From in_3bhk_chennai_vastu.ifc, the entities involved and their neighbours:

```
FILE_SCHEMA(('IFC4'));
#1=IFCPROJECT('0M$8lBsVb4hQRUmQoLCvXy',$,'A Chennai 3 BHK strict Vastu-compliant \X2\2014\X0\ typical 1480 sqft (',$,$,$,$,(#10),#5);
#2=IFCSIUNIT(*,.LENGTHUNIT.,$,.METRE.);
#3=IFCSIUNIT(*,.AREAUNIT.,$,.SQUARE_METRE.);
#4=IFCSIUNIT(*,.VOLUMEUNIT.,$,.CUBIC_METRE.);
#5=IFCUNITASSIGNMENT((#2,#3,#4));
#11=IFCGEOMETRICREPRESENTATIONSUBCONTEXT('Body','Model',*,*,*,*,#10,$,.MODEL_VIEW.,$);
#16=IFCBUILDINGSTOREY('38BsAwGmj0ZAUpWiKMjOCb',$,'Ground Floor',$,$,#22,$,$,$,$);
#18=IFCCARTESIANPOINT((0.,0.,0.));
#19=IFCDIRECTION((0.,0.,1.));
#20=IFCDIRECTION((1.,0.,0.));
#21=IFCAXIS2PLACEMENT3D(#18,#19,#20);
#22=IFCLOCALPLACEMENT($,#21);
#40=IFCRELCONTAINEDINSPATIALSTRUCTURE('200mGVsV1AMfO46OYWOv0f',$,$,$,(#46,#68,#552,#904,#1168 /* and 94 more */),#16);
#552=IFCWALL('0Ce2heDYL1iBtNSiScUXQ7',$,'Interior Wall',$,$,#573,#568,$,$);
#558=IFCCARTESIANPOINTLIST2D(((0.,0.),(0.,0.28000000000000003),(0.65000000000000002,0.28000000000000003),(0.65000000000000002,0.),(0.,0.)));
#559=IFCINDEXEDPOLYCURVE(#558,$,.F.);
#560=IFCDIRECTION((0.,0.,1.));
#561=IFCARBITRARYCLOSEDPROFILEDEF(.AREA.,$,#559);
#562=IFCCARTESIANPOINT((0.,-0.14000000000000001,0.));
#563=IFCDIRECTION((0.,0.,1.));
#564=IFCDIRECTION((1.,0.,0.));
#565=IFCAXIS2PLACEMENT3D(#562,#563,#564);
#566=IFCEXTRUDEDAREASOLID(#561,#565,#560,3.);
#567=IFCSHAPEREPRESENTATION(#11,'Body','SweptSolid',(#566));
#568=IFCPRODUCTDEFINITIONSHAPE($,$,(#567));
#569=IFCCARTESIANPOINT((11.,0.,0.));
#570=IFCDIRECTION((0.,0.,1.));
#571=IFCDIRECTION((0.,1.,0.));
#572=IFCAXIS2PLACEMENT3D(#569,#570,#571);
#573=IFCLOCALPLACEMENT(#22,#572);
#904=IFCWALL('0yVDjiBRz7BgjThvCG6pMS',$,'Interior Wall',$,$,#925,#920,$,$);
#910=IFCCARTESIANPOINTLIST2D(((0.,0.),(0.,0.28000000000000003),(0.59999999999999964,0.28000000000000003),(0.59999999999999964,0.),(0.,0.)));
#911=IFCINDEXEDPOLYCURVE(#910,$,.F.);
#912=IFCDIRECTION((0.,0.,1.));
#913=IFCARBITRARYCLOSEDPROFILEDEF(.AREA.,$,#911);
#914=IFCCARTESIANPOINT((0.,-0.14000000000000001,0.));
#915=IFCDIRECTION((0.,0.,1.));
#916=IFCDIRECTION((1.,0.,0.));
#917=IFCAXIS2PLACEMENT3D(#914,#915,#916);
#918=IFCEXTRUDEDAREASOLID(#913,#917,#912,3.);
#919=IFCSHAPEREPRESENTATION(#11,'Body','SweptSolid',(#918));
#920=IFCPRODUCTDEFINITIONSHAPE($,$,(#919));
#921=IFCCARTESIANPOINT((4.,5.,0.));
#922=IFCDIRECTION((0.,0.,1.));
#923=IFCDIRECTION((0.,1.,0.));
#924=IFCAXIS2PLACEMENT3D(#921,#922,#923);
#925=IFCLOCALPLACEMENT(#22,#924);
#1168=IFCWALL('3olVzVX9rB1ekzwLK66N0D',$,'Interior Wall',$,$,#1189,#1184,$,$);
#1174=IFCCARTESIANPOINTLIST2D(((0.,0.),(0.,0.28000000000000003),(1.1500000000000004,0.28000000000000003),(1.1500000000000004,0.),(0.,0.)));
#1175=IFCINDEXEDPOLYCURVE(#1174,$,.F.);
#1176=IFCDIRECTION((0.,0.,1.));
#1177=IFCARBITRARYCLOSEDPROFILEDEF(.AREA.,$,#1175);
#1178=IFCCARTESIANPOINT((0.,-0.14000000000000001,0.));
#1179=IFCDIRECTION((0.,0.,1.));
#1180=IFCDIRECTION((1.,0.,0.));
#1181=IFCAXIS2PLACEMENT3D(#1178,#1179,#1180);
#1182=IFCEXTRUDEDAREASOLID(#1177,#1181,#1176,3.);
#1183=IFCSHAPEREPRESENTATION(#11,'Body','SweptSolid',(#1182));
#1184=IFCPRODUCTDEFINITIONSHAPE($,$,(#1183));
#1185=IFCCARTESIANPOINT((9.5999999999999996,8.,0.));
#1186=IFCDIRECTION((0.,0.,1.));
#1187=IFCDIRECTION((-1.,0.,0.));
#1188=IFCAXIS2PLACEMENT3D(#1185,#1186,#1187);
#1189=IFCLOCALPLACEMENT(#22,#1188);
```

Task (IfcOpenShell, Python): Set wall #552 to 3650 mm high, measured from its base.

```python
import ifcopenshell
import ifcopenshell.geom
import ifcopenshell.util.representation
import ifcopenshell.util.shape
import ifcopenshell.util.unit

model = ifcopenshell.open("in_3bhk_chennai_vastu.ifc")
unit_scale = ifcopenshell.util.unit.calculate_unit_scale(model)
settings = ifcopenshell.geom.settings()


def volume(element):
    """Net volume in cubic metres, openings subtracted."""
    shape = ifcopenshell.geom.create_shape(settings, element)
    return ifcopenshell.util.shape.get_volume(shape.geometry)


wall = model.by_guid("0Ce2heDYL1iBtNSiScUXQ7")
before = volume(wall)

body = ifcopenshell.util.representation.get_representation(wall, "Model", "Body")
solid = body.Items[0]
old_height = solid.Depth
solid.Depth = 3.65 / unit_scale
after = volume(wall)

print(f"height {old_height:g} -> {solid.Depth:g}, volume {before:.3f} -> {after:.3f} m3")

model.write("in_3bhk_chennai_vastu_v2.ifc")
```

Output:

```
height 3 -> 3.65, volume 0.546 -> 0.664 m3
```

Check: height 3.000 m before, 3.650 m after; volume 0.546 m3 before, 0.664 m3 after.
